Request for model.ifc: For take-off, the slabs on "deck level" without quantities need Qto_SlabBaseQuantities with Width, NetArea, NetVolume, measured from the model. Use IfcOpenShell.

First a look at what the model holds.

```python
import ifcopenshell
import ifcopenshell.util.element
import ifcopenshell.util.unit

model = ifcopenshell.open("model.ifc")
print(model.schema)
for unit_type in ("LENGTHUNIT", "AREAUNIT", "VOLUMEUNIT"):
    print(unit_type, ifcopenshell.util.unit.calculate_unit_scale(model, unit_type))
storey = next(s for s in model.by_type("IfcBuildingStorey") if s.Name == "deck level")
slabs = [e for e in ifcopenshell.util.element.get_decomposition(storey) if e.is_a("IfcSlab")]
for e in sorted(slabs, key=lambda e: e.id()):
    print(e.id(), e.is_a(), e.Name, list(ifcopenshell.util.element.get_psets(e, qtos_only=True)), sep=" | ")
```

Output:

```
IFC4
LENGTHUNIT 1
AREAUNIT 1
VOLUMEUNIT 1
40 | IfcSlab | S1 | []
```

```python
import ifcopenshell
import ifcopenshell.api.pset
import ifcopenshell.geom
import ifcopenshell.util.element
import ifcopenshell.util.shape
import ifcopenshell.util.unit

model = ifcopenshell.open("model.ifc")
unit_scale = ifcopenshell.util.unit.calculate_unit_scale(model)
area_scale = ifcopenshell.util.unit.calculate_unit_scale(model, "AREAUNIT")
volume_scale = ifcopenshell.util.unit.calculate_unit_scale(model, "VOLUMEUNIT")
settings = ifcopenshell.geom.settings()

storey = next(s for s in model.by_type("IfcBuildingStorey") if s.Name == "deck level")
slabs = [e for e in ifcopenshell.util.element.get_decomposition(storey) if e.is_a("IfcSlab")]

for e in sorted(slabs, key=lambda e: e.id()):
    if ifcopenshell.util.element.get_psets(e, qtos_only=True, should_inherit=False):
        continue
    # Geometry comes back in metres, in the element's own axes.
    shape = ifcopenshell.geom.create_shape(settings, e)
    values = {
        "Width": ifcopenshell.util.shape.get_z(shape.geometry) / unit_scale,
        "NetArea": ifcopenshell.util.shape.get_footprint_area(shape.geometry) / area_scale,
        "NetVolume": ifcopenshell.util.shape.get_volume(shape.geometry) / volume_scale,
    }
    qto = ifcopenshell.api.pset.add_qto(model, product=e, name="Qto_SlabBaseQuantities")
    ifcopenshell.api.pset.edit_qto(model, qto=qto, properties=values)
    print(e.id(), {k: round(v, 3) for k, v in values.items()})

model.write("model-out.ifc")
```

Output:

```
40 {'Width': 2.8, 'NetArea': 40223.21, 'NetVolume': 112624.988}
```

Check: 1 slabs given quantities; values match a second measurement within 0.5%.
